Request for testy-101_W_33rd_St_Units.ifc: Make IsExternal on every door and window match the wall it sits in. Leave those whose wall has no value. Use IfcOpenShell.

First a look at what the model holds.

```python
import ifcopenshell
import ifcopenshell.util.element

model = ifcopenshell.open("testy-101_W_33rd_St_Units.ifc")
print(model.schema)
seen = {}
for e in model.by_type("IfcDoor") + model.by_type("IfcWindow"):
    if not e.FillsVoids:
        continue
    host = e.FillsVoids[0].RelatingOpeningElement.VoidsElements[0].RelatingBuildingElement
    own = ifcopenshell.util.element.get_pset(e, f"Pset_{e.is_a()[3:].removesuffix('StandardCase')}Common", "IsExternal")
    wall = ifcopenshell.util.element.get_pset(host, "Pset_WallCommon", "IsExternal")
    seen[e.is_a(), own, wall] = seen.get((e.is_a(), own, wall), 0) + 1
for (cls, own, wall), count in sorted(seen.items(), key=str):
    print(count, cls, "IsExternal:", own, "| host wall:", wall)
```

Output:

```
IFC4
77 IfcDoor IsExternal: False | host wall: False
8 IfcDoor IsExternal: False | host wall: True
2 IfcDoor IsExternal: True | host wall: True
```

```python
import ifcopenshell
import ifcopenshell.api.pset
import ifcopenshell.util.element

model = ifcopenshell.open("testy-101_W_33rd_St_Units.ifc")

count = 0
for ifc_class, pset_name in (("IfcDoor", "Pset_DoorCommon"), ("IfcWindow", "Pset_WindowCommon")):
    for e in model.by_type(ifc_class):
        if not e.FillsVoids:
            continue
        host = e.FillsVoids[0].RelatingOpeningElement.VoidsElements[0].RelatingBuildingElement
        external = ifcopenshell.util.element.get_pset(host, "Pset_WallCommon", "IsExternal")
        if external is None or ifcopenshell.util.element.get_pset(e, pset_name, "IsExternal") == external:
            continue
        pset = ifcopenshell.api.pset.add_pset(model, product=e, name=pset_name)
        ifcopenshell.api.pset.edit_pset(model, pset=pset, properties={"IsExternal": external})
        count += 1

print(count, "updated")

model.write("testy-101_W_33rd_St_Units_edited.ifc")
```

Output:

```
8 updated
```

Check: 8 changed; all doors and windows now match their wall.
